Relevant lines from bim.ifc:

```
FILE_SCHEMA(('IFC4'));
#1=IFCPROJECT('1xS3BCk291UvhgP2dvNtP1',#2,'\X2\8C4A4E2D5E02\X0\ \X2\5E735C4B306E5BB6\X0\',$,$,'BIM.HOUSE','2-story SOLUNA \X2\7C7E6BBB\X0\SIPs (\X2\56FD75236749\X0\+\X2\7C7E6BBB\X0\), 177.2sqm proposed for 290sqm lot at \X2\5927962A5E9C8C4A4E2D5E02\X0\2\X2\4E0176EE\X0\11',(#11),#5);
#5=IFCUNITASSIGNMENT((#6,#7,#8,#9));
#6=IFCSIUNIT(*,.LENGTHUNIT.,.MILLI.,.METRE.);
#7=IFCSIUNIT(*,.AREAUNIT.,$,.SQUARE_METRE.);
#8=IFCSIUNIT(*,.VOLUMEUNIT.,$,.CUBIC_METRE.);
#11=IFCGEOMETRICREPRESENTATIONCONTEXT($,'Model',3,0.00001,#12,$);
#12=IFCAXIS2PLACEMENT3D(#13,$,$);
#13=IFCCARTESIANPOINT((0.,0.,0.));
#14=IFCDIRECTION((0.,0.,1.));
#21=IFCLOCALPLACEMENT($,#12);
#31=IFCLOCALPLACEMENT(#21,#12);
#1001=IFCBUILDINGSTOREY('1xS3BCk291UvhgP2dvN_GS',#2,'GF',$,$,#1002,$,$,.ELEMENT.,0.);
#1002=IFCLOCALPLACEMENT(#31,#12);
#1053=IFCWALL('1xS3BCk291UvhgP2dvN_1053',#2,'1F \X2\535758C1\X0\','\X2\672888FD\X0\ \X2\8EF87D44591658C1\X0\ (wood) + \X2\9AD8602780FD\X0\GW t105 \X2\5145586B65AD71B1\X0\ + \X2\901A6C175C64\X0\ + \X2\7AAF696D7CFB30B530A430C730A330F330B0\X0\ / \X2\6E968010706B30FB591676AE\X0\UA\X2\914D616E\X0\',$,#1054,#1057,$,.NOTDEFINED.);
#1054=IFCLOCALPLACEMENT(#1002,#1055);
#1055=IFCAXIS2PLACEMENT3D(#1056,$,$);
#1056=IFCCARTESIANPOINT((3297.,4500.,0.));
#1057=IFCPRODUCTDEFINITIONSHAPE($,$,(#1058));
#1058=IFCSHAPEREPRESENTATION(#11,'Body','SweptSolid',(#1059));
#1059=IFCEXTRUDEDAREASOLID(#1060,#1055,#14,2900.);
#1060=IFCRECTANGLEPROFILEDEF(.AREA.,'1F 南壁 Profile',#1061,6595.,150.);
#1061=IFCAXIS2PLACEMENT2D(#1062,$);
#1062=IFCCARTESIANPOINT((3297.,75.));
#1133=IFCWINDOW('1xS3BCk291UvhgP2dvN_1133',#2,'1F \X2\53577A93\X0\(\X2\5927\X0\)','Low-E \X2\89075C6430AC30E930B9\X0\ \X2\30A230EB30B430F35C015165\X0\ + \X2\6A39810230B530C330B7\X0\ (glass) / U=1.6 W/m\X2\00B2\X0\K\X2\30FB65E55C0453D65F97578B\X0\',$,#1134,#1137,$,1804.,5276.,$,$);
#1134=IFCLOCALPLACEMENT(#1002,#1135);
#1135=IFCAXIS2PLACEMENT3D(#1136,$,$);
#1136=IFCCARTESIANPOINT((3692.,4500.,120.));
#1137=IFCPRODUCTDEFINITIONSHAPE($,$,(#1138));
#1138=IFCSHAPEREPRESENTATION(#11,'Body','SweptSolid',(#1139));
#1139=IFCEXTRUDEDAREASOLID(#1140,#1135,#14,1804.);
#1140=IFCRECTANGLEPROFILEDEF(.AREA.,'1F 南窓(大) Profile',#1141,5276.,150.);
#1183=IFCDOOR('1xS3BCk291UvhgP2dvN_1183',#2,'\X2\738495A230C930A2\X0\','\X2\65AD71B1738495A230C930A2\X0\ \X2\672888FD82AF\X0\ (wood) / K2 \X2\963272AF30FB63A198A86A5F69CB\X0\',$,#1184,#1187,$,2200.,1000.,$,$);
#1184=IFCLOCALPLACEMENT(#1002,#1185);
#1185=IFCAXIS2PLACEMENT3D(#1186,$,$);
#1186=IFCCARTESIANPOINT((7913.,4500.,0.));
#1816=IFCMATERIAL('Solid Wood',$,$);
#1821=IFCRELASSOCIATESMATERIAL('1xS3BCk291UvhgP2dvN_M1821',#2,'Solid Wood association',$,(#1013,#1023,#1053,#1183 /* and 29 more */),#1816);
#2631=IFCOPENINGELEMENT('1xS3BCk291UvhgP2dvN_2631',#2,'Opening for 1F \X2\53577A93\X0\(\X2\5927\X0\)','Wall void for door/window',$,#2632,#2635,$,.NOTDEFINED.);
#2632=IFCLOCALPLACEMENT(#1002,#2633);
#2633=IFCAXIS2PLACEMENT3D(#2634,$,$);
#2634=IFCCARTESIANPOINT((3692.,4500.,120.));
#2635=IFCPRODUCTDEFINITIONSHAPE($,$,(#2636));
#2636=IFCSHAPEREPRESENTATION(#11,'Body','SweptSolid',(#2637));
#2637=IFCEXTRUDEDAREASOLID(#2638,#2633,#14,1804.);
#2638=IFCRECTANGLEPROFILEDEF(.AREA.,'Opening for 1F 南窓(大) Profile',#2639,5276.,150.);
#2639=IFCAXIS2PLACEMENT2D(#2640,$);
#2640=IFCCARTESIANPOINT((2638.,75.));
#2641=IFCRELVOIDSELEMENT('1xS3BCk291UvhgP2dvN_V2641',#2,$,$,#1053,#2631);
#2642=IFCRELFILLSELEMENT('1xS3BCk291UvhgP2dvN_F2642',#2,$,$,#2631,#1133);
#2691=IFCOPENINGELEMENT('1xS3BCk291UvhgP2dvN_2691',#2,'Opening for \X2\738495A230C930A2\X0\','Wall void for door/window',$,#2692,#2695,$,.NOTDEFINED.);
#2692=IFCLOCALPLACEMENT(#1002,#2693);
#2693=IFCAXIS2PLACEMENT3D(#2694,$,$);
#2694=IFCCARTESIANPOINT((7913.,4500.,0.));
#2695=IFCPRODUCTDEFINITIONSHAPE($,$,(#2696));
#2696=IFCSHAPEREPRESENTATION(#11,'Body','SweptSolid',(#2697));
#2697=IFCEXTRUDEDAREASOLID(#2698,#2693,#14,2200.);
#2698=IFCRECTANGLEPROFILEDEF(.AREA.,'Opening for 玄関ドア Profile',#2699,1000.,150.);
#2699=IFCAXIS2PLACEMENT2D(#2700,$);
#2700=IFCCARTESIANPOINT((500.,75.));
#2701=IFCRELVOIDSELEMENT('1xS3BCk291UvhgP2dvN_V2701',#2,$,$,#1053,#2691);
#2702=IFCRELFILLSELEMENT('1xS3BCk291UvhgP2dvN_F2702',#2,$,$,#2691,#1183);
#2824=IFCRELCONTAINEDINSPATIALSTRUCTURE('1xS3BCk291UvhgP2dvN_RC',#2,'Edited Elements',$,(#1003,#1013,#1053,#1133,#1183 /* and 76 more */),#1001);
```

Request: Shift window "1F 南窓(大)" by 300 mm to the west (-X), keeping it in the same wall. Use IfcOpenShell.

```python
import ifcopenshell
import ifcopenshell.api.geometry
import ifcopenshell.util.placement
import ifcopenshell.util.unit

model = ifcopenshell.open("bim.ifc")
unit_scale = ifcopenshell.util.unit.calculate_unit_scale(model)

window = model.by_guid("1xS3BCk291UvhgP2dvN_1133")
opening = window.FillsVoids[0].RelatingOpeningElement
wall = opening.VoidsElements[0].RelatingBuildingElement

wall_matrix = ifcopenshell.util.placement.get_local_placement(wall.ObjectPlacement)
shift = wall_matrix[:3, 0] * -0.3 / unit_scale
before = ifcopenshell.util.placement.get_local_placement(window.ObjectPlacement)[:3, 3].copy()

# The window is not placed relative to its opening, so move both.
for product in (opening, window):
    matrix = ifcopenshell.util.placement.get_local_placement(product.ObjectPlacement)
    matrix[:3, 3] += shift
    ifcopenshell.api.geometry.edit_object_placement(model, product=product, matrix=matrix, is_si=False)

after = ifcopenshell.util.placement.get_local_placement(window.ObjectPlacement)[:3, 3]
print("window moved by", (after - before).round(3) + 0.0)

model.write("bim_v2.ifc")
```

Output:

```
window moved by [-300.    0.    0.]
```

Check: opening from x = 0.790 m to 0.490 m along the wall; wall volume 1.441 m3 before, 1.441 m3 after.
